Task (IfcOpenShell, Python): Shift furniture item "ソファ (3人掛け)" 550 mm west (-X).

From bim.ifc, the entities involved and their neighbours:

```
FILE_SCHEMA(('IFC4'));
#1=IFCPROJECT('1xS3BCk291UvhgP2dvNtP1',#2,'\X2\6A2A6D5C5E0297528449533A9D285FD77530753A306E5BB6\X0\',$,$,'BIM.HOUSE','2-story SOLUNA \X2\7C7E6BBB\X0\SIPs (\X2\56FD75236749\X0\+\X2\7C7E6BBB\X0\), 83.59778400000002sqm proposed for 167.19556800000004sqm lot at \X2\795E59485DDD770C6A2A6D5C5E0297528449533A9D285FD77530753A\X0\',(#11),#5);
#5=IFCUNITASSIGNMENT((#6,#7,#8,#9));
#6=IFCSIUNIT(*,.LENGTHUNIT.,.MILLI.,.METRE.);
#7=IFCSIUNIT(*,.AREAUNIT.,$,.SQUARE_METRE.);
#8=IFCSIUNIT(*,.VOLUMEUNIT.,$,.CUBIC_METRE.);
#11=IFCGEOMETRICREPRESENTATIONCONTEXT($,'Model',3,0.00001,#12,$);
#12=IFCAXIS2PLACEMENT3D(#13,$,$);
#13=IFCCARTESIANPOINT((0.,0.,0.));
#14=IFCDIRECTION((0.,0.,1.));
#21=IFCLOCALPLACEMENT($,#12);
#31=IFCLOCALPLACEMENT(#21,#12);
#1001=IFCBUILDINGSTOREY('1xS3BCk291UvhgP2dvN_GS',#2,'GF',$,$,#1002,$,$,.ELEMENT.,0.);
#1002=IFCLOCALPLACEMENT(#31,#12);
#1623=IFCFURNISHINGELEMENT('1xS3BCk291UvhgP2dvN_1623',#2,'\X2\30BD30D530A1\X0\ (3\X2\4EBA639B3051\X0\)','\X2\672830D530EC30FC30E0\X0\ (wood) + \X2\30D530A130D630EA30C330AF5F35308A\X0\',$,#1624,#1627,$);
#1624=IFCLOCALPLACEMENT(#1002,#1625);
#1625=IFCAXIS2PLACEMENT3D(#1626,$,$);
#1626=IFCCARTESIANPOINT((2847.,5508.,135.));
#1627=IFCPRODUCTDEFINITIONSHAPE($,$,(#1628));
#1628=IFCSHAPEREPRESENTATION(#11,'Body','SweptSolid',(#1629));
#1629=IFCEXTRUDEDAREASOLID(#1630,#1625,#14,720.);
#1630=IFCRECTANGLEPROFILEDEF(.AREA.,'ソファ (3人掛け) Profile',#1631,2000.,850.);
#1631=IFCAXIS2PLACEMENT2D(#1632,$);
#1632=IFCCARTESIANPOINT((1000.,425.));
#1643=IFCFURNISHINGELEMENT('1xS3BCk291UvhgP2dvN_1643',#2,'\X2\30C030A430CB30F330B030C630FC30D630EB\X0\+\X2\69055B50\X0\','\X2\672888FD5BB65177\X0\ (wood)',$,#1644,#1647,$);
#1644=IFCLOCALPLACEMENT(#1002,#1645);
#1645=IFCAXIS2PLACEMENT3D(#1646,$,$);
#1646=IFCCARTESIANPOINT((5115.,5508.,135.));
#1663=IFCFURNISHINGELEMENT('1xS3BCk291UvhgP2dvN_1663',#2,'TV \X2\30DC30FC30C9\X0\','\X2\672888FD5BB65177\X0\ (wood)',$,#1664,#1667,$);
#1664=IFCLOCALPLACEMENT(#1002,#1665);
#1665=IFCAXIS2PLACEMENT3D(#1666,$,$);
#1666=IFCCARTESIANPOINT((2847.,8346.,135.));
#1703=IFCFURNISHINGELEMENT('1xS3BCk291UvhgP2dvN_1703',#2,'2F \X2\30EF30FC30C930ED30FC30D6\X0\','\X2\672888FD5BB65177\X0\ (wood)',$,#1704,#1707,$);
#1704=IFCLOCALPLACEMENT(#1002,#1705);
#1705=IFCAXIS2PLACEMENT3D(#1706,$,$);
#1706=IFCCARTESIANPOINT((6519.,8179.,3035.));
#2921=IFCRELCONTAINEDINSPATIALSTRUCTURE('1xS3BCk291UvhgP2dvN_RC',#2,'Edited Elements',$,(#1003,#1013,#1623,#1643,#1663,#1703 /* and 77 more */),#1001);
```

```python
import ifcopenshell
import ifcopenshell.api.geometry
import ifcopenshell.util.placement
import ifcopenshell.util.unit

model = ifcopenshell.open("bim.ifc")
unit_scale = ifcopenshell.util.unit.calculate_unit_scale(model)

item = model.by_id(1623)
matrix = ifcopenshell.util.placement.get_local_placement(item.ObjectPlacement)
matrix[0, 3] -= 0.55 / unit_scale
ifcopenshell.api.geometry.edit_object_placement(model, product=item, matrix=matrix, is_si=False)

print(ifcopenshell.util.placement.get_local_placement(item.ObjectPlacement).round(3) + 0.0)

model.write("bim_rev.ifc")
```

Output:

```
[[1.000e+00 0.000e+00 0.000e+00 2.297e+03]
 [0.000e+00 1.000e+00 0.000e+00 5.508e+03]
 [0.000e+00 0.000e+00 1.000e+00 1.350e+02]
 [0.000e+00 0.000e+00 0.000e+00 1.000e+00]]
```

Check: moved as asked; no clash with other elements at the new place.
